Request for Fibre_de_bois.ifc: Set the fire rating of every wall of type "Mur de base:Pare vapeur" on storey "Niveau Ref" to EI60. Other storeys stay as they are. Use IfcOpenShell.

First a look at what the model holds.

```python
import ifcopenshell
import ifcopenshell.util.element

model = ifcopenshell.open("Fibre_de_bois.ifc")
print(model.schema)
storey = next(s for s in model.by_type("IfcBuildingStorey") if s.Name == "Niveau Ref")
walls = [e for e in ifcopenshell.util.element.get_decomposition(storey) if e.is_a("IfcWall")]
seen = {}
for e in walls:
    element_type = ifcopenshell.util.element.get_type(e)
    key = (element_type.Name if element_type != e and element_type else None, ifcopenshell.util.element.get_pset(e, "Pset_WallCommon", "FireRating"))
    seen[key] = seen.get(key, 0) + 1
for (name, value), count in sorted(seen.items(), key=str):
    print(count, "x", name, "|", value)
```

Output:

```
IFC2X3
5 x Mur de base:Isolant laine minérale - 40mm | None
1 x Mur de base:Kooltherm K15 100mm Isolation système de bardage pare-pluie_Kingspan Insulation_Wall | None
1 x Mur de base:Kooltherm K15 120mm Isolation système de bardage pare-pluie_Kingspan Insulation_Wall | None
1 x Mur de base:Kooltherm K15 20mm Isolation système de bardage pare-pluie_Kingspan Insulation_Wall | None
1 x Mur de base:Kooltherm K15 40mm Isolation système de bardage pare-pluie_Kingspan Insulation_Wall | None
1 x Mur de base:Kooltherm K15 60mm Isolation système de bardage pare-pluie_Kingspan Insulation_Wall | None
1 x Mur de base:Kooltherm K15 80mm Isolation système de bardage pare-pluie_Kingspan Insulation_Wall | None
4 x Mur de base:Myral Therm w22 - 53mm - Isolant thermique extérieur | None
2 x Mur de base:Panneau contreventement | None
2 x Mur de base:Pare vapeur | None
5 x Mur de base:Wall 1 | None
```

```python
import ifcopenshell
import ifcopenshell.api.pset
import ifcopenshell.util.element

model = ifcopenshell.open("Fibre_de_bois.ifc")

storey = next(s for s in model.by_type("IfcBuildingStorey") if s.Name == "Niveau Ref")
walls = [e for e in ifcopenshell.util.element.get_decomposition(storey) if e.is_a("IfcWall")]

count = 0
for e in walls:
    element_type = ifcopenshell.util.element.get_type(e)
    if element_type in (None, e) or element_type.Name != "Mur de base:Pare vapeur":
        continue
    # add_pset returns the element's existing set when there is one.
    pset = ifcopenshell.api.pset.add_pset(model, product=e, name="Pset_WallCommon")
    ifcopenshell.api.pset.edit_pset(model, pset=pset, properties={"FireRating": "EI60"})
    count += 1

print(count, "walls updated")

model.write("Fibre_de_bois_v2.ifc")
```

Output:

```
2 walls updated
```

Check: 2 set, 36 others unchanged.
